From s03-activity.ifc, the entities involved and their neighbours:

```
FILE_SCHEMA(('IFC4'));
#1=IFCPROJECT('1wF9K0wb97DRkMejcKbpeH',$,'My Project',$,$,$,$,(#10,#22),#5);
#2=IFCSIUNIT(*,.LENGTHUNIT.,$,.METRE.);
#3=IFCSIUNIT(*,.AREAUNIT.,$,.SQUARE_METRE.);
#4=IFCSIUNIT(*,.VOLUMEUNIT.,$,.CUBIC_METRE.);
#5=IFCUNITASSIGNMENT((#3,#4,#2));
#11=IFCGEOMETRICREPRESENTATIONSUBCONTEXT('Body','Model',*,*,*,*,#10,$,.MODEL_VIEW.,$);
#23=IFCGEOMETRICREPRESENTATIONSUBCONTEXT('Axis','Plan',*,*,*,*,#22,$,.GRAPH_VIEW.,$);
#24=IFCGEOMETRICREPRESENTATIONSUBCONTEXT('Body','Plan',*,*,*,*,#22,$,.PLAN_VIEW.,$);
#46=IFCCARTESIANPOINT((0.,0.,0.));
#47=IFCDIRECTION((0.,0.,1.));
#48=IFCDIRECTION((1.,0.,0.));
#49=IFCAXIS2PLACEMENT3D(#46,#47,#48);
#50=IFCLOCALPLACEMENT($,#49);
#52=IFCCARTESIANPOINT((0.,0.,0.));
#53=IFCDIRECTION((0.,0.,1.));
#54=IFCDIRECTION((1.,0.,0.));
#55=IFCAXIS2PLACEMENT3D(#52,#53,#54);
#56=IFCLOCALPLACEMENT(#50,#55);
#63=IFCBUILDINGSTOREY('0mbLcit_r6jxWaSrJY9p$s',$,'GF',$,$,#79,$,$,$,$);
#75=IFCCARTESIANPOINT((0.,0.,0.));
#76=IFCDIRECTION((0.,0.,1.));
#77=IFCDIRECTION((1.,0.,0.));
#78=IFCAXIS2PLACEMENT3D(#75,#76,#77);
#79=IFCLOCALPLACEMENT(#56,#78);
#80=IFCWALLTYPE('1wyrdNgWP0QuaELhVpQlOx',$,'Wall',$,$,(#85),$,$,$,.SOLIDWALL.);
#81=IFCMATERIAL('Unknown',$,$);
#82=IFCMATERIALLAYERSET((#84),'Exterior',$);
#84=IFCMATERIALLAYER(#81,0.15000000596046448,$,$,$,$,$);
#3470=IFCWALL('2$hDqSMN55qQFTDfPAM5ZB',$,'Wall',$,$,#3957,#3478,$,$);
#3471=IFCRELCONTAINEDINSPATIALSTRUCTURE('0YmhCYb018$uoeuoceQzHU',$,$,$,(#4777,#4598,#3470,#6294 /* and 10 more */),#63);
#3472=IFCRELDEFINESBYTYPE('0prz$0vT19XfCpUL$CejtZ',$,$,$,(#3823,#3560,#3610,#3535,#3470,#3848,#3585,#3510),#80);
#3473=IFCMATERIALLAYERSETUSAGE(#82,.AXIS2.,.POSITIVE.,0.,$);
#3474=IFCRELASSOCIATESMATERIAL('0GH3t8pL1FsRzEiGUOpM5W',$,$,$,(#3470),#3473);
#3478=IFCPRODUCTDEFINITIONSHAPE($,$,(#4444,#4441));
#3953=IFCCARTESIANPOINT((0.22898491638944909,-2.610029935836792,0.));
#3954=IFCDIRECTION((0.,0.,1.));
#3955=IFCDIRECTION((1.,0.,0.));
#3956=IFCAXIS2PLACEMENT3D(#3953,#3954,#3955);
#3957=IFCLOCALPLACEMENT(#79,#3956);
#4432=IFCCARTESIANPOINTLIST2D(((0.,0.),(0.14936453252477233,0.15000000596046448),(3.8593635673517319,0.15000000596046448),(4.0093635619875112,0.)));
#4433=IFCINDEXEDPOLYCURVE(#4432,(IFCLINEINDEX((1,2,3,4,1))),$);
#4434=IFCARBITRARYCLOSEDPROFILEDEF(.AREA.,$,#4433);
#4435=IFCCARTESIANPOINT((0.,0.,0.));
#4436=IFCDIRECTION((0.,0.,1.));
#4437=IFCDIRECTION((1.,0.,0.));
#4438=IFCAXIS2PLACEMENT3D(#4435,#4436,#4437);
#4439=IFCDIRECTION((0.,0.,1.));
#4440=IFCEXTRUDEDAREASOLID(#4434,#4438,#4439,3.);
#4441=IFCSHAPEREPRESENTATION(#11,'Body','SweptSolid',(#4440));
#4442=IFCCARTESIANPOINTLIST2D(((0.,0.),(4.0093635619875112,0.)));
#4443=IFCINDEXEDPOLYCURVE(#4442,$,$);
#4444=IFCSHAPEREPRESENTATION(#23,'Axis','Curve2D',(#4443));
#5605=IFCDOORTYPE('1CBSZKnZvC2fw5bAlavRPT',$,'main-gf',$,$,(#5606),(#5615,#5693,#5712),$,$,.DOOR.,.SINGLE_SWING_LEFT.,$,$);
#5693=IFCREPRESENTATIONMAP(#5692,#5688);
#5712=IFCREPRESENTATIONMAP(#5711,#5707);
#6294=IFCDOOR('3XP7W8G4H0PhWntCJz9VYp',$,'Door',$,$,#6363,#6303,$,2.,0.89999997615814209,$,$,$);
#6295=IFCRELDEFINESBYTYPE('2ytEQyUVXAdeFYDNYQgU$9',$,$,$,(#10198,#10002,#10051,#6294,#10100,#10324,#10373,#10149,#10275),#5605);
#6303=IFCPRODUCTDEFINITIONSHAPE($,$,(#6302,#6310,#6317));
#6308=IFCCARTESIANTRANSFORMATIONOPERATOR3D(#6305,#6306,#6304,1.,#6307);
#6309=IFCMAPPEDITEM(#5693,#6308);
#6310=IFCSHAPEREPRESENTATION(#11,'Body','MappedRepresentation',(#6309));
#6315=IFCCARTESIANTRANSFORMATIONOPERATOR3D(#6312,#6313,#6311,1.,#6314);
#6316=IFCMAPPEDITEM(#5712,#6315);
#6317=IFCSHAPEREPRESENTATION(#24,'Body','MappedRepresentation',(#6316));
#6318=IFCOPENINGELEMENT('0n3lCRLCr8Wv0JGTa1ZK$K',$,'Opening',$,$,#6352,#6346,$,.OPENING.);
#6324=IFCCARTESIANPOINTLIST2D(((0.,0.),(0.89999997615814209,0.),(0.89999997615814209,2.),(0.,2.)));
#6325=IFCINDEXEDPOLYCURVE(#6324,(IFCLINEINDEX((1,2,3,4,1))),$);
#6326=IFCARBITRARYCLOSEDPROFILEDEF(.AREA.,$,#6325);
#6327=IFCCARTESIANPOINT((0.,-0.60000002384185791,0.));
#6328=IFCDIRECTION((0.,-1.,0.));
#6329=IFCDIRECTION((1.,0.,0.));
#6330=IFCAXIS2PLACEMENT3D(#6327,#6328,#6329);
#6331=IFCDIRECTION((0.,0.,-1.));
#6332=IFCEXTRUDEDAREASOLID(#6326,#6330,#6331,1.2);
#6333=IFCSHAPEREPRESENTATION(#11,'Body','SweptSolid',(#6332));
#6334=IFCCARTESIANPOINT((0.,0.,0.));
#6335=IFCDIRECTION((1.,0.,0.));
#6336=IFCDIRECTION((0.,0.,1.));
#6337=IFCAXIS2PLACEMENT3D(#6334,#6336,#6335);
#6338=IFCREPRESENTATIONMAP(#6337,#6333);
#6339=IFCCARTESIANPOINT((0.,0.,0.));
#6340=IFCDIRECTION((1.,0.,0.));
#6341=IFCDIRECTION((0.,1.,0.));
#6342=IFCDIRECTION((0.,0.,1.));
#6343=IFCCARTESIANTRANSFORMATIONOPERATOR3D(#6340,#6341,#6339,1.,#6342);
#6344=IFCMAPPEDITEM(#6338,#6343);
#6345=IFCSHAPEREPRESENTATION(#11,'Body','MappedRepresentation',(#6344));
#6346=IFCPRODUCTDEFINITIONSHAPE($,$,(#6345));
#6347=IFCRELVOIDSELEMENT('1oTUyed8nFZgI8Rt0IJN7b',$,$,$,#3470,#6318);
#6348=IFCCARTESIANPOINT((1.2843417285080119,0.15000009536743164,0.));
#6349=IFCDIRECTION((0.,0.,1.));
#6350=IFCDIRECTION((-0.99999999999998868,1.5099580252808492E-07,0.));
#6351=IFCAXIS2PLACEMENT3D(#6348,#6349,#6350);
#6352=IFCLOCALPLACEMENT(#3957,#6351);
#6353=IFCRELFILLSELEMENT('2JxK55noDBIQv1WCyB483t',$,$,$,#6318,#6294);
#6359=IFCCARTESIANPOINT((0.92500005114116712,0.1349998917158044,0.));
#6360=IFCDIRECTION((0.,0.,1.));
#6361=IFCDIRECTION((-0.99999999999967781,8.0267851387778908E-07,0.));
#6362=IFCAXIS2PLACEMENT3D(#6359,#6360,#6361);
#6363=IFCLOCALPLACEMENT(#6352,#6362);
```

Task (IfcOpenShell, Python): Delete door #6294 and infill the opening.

```python
import ifcopenshell
import ifcopenshell.api.feature
import ifcopenshell.api.root
import ifcopenshell.geom
import ifcopenshell.util.shape

model = ifcopenshell.open("s03-activity.ifc")
settings = ifcopenshell.geom.settings()


def volume(element):
    """Net volume in cubic metres, openings subtracted."""
    shape = ifcopenshell.geom.create_shape(settings, element)
    return ifcopenshell.util.shape.get_volume(shape.geometry)


door = model.by_guid("3XP7W8G4H0PhWntCJz9VYp")
opening = door.FillsVoids[0].RelatingOpeningElement
wall = opening.VoidsElements[0].RelatingBuildingElement
before = volume(wall)

ifcopenshell.api.root.remove_product(model, product=door)
ifcopenshell.api.feature.remove_feature(model, feature=opening)

after = volume(wall)

print(f"wall volume {before:.3f} -> {after:.3f} m3")

model.write("s03-activity_v2.ifc")
```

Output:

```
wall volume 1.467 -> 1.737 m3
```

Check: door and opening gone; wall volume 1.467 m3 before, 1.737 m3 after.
